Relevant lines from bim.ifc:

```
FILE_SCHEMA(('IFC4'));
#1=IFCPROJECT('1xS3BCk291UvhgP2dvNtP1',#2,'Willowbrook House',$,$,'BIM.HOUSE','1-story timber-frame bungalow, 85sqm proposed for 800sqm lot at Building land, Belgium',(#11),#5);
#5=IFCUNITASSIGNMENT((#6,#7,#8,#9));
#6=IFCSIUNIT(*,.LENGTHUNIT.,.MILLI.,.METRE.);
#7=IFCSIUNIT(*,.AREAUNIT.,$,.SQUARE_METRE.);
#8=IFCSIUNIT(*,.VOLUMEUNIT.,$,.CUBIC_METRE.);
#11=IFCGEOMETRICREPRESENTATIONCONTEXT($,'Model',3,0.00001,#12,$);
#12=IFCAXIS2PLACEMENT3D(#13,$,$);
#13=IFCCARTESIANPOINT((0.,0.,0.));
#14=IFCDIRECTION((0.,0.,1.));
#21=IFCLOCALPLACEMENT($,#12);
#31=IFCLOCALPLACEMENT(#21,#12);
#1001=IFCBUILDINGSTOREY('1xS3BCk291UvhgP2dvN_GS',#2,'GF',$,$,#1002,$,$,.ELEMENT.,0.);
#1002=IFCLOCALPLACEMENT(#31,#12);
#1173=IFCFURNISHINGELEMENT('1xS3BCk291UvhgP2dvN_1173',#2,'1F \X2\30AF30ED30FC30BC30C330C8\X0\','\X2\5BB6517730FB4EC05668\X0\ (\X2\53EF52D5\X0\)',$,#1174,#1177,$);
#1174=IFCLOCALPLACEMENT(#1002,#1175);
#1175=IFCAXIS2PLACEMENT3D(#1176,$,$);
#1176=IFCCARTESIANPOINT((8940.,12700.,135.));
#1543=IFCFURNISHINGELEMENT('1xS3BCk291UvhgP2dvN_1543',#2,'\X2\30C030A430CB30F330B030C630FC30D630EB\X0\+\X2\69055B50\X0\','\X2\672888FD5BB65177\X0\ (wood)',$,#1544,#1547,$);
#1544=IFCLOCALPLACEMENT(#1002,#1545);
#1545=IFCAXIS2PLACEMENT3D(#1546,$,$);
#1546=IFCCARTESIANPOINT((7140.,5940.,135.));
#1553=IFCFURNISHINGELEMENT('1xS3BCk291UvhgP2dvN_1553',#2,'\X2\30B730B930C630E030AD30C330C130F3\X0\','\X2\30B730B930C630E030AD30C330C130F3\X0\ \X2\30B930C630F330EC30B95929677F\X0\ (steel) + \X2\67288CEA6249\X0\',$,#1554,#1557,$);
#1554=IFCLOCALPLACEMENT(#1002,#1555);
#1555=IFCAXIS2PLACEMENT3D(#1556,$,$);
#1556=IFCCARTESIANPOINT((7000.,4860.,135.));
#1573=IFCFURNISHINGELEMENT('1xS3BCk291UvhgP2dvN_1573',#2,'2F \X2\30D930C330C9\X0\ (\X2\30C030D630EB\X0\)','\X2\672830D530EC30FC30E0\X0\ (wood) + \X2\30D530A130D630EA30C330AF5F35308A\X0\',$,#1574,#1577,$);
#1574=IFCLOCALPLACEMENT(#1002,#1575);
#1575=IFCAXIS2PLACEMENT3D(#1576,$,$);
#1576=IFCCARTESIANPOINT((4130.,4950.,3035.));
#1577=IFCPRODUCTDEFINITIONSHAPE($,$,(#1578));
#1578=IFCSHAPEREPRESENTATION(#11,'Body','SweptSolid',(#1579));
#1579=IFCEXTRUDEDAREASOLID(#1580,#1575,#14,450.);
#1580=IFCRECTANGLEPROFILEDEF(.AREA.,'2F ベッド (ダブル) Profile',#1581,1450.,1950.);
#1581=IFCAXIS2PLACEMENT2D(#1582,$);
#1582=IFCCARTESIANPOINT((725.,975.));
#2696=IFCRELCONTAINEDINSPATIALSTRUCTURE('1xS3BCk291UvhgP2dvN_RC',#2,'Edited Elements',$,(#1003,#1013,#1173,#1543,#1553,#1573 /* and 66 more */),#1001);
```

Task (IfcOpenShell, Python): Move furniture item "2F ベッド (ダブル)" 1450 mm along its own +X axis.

```python
import ifcopenshell
import ifcopenshell.api.geometry
import ifcopenshell.util.placement

model = ifcopenshell.open("bim.ifc")

item = model.by_id(1573)
matrix = ifcopenshell.util.placement.get_local_placement(item.ObjectPlacement)
matrix[:3, 3] += matrix[:3, 0] * 1450.0
ifcopenshell.api.geometry.edit_object_placement(model, product=item, matrix=matrix, is_si=False)

print(ifcopenshell.util.placement.get_local_placement(item.ObjectPlacement).round(3) + 0.0)

model.write("bim_updated.ifc")
```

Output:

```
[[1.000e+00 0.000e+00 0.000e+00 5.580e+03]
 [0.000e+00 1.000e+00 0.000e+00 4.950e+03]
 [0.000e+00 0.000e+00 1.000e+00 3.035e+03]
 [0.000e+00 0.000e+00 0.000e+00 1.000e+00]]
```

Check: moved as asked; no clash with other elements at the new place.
